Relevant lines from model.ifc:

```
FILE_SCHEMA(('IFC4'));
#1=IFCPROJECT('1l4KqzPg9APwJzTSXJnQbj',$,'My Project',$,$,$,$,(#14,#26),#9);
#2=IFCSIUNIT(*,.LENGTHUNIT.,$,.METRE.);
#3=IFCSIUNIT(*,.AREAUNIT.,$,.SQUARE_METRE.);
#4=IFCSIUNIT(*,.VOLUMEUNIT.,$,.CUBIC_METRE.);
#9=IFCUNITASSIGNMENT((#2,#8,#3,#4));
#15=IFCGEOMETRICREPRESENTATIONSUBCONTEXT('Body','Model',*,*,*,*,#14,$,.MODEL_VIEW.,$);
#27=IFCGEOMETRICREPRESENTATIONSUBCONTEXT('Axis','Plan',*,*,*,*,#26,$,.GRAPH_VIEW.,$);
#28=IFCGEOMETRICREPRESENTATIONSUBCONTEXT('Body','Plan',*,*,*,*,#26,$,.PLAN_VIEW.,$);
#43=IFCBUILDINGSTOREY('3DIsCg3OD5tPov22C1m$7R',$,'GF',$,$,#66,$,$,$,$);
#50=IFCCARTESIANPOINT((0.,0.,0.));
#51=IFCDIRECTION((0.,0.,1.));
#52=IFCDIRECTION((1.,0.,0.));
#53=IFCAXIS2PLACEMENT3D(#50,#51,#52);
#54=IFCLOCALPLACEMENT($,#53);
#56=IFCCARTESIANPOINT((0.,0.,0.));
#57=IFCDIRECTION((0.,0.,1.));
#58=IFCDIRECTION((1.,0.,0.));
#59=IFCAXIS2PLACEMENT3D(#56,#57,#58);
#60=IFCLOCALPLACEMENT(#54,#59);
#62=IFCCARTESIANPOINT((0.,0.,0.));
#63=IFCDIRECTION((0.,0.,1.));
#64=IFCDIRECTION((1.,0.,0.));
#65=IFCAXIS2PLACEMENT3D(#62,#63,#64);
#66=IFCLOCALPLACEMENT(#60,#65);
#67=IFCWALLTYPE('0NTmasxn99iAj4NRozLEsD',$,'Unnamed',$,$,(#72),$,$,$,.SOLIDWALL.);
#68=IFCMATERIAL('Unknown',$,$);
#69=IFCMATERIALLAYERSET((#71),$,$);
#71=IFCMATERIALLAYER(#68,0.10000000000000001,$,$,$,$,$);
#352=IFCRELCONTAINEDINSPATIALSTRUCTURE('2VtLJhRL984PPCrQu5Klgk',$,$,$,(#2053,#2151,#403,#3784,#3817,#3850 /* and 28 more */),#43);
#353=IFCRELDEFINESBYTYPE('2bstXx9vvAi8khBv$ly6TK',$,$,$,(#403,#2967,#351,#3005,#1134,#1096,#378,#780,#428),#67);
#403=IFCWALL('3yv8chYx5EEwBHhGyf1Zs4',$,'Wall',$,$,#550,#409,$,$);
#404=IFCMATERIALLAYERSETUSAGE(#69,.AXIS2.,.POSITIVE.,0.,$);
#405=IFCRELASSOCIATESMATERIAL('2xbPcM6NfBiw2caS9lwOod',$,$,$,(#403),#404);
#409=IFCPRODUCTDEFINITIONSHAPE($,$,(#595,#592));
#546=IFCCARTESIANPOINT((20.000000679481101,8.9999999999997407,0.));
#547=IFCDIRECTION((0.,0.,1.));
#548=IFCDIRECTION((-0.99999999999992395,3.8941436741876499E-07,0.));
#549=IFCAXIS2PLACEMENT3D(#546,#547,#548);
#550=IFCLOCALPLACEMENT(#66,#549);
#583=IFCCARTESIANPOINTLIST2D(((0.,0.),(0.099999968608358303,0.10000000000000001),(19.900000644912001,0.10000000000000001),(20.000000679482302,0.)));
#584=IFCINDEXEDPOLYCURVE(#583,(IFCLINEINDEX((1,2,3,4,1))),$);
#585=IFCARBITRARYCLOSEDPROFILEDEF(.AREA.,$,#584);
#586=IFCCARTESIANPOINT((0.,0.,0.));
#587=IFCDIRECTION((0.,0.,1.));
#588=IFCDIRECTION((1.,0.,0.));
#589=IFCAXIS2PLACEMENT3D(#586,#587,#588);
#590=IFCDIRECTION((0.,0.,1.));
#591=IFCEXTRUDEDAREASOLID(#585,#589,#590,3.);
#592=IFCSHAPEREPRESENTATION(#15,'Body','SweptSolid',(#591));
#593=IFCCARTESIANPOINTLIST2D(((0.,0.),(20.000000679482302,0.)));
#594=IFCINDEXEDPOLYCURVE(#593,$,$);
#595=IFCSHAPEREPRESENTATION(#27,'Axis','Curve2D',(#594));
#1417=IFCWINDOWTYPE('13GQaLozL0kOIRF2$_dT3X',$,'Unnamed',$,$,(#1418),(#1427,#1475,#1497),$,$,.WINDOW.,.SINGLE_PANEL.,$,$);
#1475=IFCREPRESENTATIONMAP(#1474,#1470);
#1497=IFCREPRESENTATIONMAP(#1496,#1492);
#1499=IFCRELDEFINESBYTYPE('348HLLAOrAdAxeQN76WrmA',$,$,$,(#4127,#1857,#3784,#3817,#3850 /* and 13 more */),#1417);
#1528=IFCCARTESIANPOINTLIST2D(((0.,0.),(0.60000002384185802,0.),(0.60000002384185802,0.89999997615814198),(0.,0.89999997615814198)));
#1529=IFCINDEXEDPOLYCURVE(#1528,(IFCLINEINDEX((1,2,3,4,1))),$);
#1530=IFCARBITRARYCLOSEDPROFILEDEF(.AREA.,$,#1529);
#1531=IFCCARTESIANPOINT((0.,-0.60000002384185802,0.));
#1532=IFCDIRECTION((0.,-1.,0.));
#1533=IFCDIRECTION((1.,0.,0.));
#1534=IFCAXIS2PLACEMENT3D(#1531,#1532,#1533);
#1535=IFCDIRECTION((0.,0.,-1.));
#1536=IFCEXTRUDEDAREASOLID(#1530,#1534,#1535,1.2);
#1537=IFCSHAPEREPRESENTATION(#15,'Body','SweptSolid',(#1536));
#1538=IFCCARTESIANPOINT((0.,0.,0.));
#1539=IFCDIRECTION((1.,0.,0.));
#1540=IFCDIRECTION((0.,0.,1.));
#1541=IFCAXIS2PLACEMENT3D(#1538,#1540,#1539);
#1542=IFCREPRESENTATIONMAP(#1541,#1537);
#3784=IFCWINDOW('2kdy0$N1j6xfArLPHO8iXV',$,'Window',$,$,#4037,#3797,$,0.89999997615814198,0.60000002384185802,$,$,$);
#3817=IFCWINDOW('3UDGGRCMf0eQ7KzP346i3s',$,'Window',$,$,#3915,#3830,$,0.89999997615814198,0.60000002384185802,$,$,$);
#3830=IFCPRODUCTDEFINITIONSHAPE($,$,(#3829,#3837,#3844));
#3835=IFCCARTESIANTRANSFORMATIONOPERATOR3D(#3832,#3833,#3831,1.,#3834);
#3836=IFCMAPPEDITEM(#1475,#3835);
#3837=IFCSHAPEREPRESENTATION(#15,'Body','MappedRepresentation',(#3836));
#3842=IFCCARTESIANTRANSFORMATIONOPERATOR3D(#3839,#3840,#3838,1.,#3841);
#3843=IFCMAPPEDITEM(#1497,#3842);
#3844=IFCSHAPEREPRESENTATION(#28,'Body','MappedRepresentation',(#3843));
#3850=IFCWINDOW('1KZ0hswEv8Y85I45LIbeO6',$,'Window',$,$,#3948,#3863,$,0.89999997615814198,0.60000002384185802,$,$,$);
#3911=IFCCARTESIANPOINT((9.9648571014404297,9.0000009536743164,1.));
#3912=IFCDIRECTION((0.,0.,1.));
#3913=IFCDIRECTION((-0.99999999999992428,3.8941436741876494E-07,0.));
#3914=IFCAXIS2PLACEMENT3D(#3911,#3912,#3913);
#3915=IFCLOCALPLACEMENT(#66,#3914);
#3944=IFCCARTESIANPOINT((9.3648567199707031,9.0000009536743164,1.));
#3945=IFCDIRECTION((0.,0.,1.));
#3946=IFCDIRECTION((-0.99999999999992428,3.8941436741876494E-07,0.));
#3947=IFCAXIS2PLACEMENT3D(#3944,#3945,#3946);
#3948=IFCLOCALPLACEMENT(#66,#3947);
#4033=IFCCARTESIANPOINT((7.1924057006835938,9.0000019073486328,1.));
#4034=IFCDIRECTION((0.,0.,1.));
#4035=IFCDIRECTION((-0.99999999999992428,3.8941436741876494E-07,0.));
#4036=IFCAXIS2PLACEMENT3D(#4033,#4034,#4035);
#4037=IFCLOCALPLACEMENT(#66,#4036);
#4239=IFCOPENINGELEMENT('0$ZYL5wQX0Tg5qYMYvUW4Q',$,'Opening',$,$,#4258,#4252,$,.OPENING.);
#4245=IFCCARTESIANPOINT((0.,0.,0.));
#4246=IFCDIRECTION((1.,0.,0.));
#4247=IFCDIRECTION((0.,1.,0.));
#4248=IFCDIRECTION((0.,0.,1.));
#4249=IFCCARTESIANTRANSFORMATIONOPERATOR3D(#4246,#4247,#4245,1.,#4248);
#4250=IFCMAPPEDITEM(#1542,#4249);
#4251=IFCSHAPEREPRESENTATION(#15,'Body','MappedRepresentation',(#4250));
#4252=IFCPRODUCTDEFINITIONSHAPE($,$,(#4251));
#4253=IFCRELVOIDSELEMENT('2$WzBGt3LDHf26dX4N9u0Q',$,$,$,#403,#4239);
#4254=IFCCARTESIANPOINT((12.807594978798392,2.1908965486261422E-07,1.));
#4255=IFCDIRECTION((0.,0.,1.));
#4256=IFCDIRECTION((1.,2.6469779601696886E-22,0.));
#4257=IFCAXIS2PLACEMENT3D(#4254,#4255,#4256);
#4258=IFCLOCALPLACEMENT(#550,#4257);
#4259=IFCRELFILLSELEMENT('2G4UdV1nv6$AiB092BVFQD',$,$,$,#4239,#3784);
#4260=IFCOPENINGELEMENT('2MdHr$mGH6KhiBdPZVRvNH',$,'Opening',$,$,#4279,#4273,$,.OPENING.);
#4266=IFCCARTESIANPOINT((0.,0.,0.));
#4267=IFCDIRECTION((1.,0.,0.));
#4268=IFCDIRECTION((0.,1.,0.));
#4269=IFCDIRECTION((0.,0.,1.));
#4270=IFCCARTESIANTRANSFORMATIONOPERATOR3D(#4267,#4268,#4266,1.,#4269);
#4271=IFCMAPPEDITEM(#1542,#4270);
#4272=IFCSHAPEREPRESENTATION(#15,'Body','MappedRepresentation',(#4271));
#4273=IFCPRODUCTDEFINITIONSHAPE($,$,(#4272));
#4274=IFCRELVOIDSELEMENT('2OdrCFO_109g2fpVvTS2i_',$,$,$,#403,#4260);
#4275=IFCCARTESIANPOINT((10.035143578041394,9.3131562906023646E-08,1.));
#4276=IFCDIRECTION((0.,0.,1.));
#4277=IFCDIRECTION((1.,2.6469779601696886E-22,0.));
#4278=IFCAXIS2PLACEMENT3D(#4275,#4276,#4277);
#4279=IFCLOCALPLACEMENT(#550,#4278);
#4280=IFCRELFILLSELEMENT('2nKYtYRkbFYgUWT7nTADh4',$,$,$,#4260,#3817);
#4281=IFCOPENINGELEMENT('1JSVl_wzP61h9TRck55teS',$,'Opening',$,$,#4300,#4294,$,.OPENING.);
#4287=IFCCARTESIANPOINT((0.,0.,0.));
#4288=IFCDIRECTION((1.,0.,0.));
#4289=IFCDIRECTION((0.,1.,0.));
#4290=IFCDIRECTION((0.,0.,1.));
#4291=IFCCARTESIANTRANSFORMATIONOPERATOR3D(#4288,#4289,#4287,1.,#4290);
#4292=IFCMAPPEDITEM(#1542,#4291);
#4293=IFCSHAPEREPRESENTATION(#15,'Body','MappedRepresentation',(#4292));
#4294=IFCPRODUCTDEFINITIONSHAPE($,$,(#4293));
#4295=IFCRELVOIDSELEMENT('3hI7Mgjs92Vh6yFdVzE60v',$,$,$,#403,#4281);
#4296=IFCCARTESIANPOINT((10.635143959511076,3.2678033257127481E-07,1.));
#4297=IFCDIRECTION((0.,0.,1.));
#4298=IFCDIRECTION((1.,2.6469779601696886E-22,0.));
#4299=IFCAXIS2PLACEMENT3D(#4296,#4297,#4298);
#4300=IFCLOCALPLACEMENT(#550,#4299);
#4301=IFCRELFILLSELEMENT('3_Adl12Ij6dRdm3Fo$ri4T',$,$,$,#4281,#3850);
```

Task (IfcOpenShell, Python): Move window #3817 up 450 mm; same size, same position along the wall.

```python
import numpy as np
import ifcopenshell
import ifcopenshell.api.geometry
import ifcopenshell.util.placement
import ifcopenshell.util.unit

model = ifcopenshell.open("model.ifc")
unit_scale = ifcopenshell.util.unit.calculate_unit_scale(model)

window = model.by_guid("3UDGGRCMf0eQ7KzP346i3s")
opening = window.FillsVoids[0].RelatingOpeningElement
dz = 0.45

shift = np.array([0.0, 0.0, dz])
# The window is not placed relative to its opening, so move both.
for product in (opening, window):
    matrix = ifcopenshell.util.placement.get_local_placement(product.ObjectPlacement)
    matrix[:3, 3] += shift
    ifcopenshell.api.geometry.edit_object_placement(model, product=product, matrix=matrix, is_si=False)

print(f"moved by {dz * unit_scale:+.3f} m")

model.write("model_edited.ifc")
```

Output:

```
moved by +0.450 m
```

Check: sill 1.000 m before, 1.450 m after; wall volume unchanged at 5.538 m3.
